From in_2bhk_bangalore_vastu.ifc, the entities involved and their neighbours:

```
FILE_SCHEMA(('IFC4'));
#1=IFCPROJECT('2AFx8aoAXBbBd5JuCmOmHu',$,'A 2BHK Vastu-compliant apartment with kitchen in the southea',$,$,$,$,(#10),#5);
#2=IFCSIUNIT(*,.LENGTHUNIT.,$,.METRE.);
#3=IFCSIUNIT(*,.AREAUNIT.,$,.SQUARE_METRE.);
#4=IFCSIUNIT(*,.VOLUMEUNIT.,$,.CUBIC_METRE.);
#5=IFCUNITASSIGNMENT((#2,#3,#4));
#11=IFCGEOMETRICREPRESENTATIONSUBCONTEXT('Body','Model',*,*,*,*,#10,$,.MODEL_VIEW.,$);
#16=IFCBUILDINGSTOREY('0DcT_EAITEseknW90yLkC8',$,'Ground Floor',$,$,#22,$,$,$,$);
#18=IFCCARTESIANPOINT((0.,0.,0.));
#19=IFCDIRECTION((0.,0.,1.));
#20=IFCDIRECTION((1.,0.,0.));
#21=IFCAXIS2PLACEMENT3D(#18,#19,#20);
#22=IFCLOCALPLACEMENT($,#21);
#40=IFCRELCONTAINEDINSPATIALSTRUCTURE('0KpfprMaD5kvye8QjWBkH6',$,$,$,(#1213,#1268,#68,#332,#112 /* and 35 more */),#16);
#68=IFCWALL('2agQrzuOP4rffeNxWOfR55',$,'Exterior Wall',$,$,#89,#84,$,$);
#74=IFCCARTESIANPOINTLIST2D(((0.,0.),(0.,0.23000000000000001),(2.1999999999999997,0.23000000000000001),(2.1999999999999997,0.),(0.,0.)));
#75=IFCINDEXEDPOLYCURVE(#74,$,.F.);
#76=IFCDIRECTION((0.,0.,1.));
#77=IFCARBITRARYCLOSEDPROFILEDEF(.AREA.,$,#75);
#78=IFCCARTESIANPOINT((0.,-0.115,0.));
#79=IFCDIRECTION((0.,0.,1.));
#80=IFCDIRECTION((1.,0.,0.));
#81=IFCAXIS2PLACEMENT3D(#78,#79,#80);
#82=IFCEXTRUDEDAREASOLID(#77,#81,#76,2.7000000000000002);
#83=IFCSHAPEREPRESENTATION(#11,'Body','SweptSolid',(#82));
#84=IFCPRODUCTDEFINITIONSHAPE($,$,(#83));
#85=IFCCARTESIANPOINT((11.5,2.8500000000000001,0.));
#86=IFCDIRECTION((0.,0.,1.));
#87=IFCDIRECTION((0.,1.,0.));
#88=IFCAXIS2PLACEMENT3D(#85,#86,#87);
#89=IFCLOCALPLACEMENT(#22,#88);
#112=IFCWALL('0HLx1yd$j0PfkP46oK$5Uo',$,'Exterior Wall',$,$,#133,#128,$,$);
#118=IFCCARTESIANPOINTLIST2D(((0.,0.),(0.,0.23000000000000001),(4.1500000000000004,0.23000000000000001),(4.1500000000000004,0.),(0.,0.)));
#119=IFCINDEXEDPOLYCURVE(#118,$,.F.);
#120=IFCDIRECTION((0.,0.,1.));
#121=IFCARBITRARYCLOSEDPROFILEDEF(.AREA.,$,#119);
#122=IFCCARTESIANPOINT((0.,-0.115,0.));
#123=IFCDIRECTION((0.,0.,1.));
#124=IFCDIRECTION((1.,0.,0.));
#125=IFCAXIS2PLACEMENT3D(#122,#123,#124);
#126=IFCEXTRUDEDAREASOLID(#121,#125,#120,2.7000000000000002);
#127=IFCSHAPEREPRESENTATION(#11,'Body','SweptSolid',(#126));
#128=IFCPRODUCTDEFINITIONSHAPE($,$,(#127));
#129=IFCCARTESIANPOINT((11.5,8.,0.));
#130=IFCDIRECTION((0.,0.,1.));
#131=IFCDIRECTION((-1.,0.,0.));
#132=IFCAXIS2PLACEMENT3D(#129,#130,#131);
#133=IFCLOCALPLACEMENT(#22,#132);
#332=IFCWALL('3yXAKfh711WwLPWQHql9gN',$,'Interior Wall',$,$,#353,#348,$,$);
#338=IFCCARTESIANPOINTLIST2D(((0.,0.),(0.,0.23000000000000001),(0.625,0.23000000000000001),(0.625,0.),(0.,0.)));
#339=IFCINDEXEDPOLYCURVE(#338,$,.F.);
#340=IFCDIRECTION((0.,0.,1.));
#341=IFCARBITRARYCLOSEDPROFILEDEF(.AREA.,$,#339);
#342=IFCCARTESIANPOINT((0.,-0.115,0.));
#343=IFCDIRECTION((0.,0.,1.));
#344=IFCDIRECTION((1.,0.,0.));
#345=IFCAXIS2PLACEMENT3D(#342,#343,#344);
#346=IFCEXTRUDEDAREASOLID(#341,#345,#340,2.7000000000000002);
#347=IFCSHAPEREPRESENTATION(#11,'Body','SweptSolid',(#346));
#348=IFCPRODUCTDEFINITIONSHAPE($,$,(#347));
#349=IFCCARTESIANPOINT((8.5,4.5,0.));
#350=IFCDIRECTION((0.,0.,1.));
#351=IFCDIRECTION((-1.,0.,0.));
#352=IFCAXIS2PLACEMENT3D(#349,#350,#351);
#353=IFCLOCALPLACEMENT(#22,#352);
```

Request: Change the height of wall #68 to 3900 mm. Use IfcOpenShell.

```python
import ifcopenshell
import ifcopenshell.geom
import ifcopenshell.util.representation
import ifcopenshell.util.shape

model = ifcopenshell.open("in_2bhk_bangalore_vastu.ifc")
settings = ifcopenshell.geom.settings()


def volume(element):
    """Net volume in cubic metres, openings subtracted."""
    shape = ifcopenshell.geom.create_shape(settings, element)
    return ifcopenshell.util.shape.get_volume(shape.geometry)


wall = model.by_id(68)
before = volume(wall)

body = ifcopenshell.util.representation.get_representation(wall, "Model", "Body")
solid = body.Items[0]
old_height = solid.Depth
solid.Depth = 3.9
after = volume(wall)

print(f"height {old_height:g} -> {solid.Depth:g}, volume {before:.3f} -> {after:.3f} m3")

model.write("in_2bhk_bangalore_vastu_rev.ifc")
```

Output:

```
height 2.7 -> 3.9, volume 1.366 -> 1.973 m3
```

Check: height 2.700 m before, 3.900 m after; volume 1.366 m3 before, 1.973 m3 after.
